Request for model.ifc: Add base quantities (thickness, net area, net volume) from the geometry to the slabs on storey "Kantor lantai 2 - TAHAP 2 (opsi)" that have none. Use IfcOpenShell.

First a look at what the model holds.

```python
import ifcopenshell
import ifcopenshell.util.element
import ifcopenshell.util.unit

model = ifcopenshell.open("model.ifc")
print(model.schema)
for unit_type in ("LENGTHUNIT", "AREAUNIT", "VOLUMEUNIT"):
    print(unit_type, ifcopenshell.util.unit.calculate_unit_scale(model, unit_type))
storey = next(s for s in model.by_type("IfcBuildingStorey") if s.Name == "Kantor lantai 2 - TAHAP 2 (opsi)")
slabs = [e for e in ifcopenshell.util.element.get_decomposition(storey) if e.is_a("IfcSlab")]
for e in sorted(slabs, key=lambda e: e.id()):
    print(e.id(), e.is_a(), e.Name, list(ifcopenshell.util.element.get_psets(e, qtos_only=True)), sep=" | ")
```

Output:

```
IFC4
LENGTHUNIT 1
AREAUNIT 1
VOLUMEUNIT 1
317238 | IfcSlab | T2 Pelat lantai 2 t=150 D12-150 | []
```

```python
import ifcopenshell
import ifcopenshell.api.pset
import ifcopenshell.geom
import ifcopenshell.util.element
import ifcopenshell.util.shape
import ifcopenshell.util.unit

model = ifcopenshell.open("model.ifc")
unit_scale = ifcopenshell.util.unit.calculate_unit_scale(model)
area_scale = ifcopenshell.util.unit.calculate_unit_scale(model, "AREAUNIT")
volume_scale = ifcopenshell.util.unit.calculate_unit_scale(model, "VOLUMEUNIT")
settings = ifcopenshell.geom.settings()

storey = next(s for s in model.by_type("IfcBuildingStorey") if s.Name == "Kantor lantai 2 - TAHAP 2 (opsi)")
slabs = [e for e in ifcopenshell.util.element.get_decomposition(storey) if e.is_a("IfcSlab")]

for e in sorted(slabs, key=lambda e: e.id()):
    if ifcopenshell.util.element.get_psets(e, qtos_only=True, should_inherit=False):
        continue
    # Geometry comes back in metres, in the element's own axes.
    shape = ifcopenshell.geom.create_shape(settings, e)
    values = {
        "Width": ifcopenshell.util.shape.get_z(shape.geometry) / unit_scale,
        "NetArea": ifcopenshell.util.shape.get_footprint_area(shape.geometry) / area_scale,
        "NetVolume": ifcopenshell.util.shape.get_volume(shape.geometry) / volume_scale,
    }
    qto = ifcopenshell.api.pset.add_qto(model, product=e, name="Qto_SlabBaseQuantities")
    ifcopenshell.api.pset.edit_qto(model, qto=qto, properties=values)
    print(e.id(), {k: round(v, 3) for k, v in values.items()})

model.write("model_v2.ifc")
```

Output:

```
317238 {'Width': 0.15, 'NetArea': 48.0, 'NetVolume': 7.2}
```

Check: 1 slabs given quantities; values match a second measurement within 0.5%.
